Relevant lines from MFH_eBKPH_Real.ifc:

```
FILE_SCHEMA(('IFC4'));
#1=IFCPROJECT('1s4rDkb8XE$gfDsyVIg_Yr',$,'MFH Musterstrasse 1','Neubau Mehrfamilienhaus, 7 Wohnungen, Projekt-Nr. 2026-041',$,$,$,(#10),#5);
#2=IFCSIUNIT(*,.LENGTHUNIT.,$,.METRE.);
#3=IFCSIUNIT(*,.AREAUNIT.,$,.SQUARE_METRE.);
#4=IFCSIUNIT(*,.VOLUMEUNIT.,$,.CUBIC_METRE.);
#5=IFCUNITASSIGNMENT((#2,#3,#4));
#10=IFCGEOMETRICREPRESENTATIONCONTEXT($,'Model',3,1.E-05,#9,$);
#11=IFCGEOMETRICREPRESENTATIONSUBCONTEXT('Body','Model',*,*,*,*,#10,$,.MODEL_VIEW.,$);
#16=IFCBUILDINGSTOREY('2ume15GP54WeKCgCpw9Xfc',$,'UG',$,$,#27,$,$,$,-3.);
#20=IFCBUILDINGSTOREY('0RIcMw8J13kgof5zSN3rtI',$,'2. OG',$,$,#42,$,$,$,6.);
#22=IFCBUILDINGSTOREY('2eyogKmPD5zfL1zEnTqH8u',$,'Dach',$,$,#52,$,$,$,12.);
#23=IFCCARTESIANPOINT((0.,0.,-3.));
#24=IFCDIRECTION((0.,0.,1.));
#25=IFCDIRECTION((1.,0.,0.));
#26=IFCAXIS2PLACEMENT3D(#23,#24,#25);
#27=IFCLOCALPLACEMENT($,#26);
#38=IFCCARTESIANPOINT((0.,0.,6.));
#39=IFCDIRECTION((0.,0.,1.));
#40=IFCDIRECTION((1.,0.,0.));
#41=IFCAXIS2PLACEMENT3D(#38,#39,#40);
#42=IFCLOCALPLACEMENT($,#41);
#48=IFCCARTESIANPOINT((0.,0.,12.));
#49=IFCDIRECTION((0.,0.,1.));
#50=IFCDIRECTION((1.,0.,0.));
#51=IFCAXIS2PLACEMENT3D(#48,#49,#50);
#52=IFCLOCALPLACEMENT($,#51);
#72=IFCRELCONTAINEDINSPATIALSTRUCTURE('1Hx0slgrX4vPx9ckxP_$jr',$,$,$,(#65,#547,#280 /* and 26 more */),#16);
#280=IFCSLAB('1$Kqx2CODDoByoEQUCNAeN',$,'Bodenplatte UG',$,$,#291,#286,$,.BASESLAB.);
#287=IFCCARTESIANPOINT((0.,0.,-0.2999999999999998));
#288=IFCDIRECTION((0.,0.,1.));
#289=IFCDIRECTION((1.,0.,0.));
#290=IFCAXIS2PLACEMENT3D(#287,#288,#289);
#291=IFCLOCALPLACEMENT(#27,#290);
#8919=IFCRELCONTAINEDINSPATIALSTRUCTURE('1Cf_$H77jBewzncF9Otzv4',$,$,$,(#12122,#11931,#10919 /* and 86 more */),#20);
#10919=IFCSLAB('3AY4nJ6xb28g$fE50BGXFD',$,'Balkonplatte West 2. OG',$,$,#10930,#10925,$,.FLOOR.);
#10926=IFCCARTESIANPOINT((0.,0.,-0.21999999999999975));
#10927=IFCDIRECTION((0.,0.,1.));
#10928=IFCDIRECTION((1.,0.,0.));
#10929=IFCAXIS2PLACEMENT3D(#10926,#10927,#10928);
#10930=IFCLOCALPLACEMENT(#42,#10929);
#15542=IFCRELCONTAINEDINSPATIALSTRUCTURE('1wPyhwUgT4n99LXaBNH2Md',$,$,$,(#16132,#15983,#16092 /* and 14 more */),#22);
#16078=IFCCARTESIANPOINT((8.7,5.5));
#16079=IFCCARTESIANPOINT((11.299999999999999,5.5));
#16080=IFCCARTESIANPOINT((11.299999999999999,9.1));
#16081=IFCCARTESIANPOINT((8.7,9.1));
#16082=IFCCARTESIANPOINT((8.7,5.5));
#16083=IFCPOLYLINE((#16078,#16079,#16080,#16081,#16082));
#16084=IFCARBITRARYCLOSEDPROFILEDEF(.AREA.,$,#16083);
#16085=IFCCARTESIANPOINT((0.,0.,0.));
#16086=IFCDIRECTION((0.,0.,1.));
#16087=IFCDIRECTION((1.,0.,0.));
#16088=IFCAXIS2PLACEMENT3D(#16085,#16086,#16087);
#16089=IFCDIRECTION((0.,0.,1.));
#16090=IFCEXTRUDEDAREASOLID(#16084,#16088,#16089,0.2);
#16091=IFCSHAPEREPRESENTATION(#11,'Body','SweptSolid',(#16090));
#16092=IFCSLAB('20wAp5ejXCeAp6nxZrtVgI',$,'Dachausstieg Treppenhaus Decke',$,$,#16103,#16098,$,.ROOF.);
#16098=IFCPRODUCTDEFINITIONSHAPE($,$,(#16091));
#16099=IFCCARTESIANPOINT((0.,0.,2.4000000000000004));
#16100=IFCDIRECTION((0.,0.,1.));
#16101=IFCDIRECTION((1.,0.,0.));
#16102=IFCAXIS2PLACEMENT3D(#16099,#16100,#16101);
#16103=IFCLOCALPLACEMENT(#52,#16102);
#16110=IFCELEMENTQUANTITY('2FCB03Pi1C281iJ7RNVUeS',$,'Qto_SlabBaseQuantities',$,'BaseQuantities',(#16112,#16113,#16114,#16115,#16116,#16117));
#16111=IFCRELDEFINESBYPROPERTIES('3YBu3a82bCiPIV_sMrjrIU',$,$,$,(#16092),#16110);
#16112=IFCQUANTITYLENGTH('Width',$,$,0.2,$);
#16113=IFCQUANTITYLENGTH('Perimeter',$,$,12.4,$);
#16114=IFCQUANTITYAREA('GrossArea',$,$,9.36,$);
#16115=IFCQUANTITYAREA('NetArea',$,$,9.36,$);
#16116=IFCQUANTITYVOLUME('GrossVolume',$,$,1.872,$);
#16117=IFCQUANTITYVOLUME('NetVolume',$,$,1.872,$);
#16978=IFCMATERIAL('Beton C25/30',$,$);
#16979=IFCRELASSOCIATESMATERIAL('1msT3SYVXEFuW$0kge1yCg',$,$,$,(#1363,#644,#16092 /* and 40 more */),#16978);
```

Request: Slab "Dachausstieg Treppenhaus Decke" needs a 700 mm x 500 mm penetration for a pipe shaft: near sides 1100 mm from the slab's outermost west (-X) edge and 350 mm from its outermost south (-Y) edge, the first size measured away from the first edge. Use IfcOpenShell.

```python
import numpy as np
import ifcopenshell
import ifcopenshell.api.feature
import ifcopenshell.api.geometry
import ifcopenshell.api.pset
import ifcopenshell.api.root
import ifcopenshell.geom
import ifcopenshell.util.element
import ifcopenshell.util.placement
import ifcopenshell.util.representation
import ifcopenshell.util.shape
import ifcopenshell.util.unit

model = ifcopenshell.open("MFH_eBKPH_Real.ifc")
unit_scale = ifcopenshell.util.unit.calculate_unit_scale(model)
area_scale = ifcopenshell.util.unit.calculate_unit_scale(model, "AREAUNIT")
volume_scale = ifcopenshell.util.unit.calculate_unit_scale(model, "VOLUMEUNIT")
settings = ifcopenshell.geom.settings()


def volume(element):
    """Net volume in cubic metres, openings subtracted."""
    shape = ifcopenshell.geom.create_shape(settings, element)
    return ifcopenshell.util.shape.get_volume(shape.geometry)


slab = model.by_id(16092)
before = volume(slab)

# Extent in the slab's own axes, in metres. The edges named are its -X and -Y sides.
slab_shape = ifcopenshell.geom.create_shape(settings, slab)
vertices = ifcopenshell.util.shape.get_vertices(slab_shape.geometry)
x_min, y_min, bottom = vertices.min(axis=0)
top = vertices[:, 2].max()

opening = ifcopenshell.api.root.create_entity(model, ifc_class="IfcOpeningElement", name="Pipe shaft opening", predefined_type="OPENING")
context = ifcopenshell.util.representation.get_context(model, "Model", "Body", "MODEL_VIEW")
width, depth = 0.7, 0.5
outline = [(0.0, 0.0), (width, 0.0), (width, depth), (0.0, depth), (0.0, 0.0)]
# Overshoot both faces by 50 mm so the cut is clean.
shape = ifcopenshell.api.geometry.add_slab_representation(
    model, context=context, depth=top - bottom + 0.1, polyline=outline
)
ifcopenshell.api.geometry.assign_representation(model, product=opening, representation=shape)

matrix = ifcopenshell.util.placement.get_local_placement(slab.ObjectPlacement)
matrix[:, 3] = matrix @ np.append(np.array([x_min + 1.1, y_min + 0.35, bottom - 0.05]) / unit_scale, 1.0)
ifcopenshell.api.geometry.edit_object_placement(model, product=opening, matrix=matrix, is_si=False)
ifcopenshell.api.feature.add_feature(model, feature=opening, element=slab)

after = volume(slab)

# Update the slab's stored quantities.
qto = model.by_id(ifcopenshell.util.element.get_pset(slab, "Qto_SlabBaseQuantities", should_inherit=False)["id"])
ifcopenshell.api.pset.edit_qto(model, qto=qto, properties={
    "NetArea": after / (top - bottom) / area_scale,
    "NetVolume": after / volume_scale,
})

print(f"slab volume {before:.3f} -> {after:.3f} m3")

model.write("MFH_eBKPH_Real_rev.ifc")
```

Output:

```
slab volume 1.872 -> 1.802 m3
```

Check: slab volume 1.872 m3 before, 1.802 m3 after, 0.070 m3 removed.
